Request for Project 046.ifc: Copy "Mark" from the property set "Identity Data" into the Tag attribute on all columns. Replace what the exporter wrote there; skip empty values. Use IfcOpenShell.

First a look at what the model holds.

```python
import ifcopenshell
import ifcopenshell.util.element

model = ifcopenshell.open("Project 046.ifc")
print(model.schema)
columns = model.by_type("IfcColumn")
print(len(columns), "columns")
for e in columns[:8]:
    source = ifcopenshell.util.element.get_pset(e, "Identity Data", "Mark")
    target = e.Tag
    print(e.id(), repr(source), repr(target), sep=" | ")
```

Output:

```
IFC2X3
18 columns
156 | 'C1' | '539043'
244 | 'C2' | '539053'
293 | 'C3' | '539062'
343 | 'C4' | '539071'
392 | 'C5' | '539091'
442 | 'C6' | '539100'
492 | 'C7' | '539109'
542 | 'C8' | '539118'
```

```python
import ifcopenshell
import ifcopenshell.util.element

model = ifcopenshell.open("Project 046.ifc")

count = 0
for e in model.by_type("IfcColumn"):
    value = ifcopenshell.util.element.get_pset(e, "Identity Data", "Mark")
    current = e.Tag
    if not value or not value.strip() or current == value:
        continue
    e.Tag = value
    count += 1

print(count, "columns updated")

model.write("Project 046_edited.ifc")
```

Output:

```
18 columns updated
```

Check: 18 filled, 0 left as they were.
